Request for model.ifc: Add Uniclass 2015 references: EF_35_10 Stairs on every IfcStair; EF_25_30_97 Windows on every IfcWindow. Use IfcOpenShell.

First a look at what the model holds.

```python
import ifcopenshell

model = ifcopenshell.open("model.ifc")
print(model.schema)
print("classifications:", [c.Name for c in model.by_type("IfcClassification")])
for ifc_class in ("IfcDoor", "IfcRoof", "IfcStair", "IfcWall", "IfcWindow"):
    print(ifc_class, len(model.by_type(ifc_class)))
```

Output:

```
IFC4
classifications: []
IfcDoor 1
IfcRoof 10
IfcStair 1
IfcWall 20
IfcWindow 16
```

```python
import ifcopenshell
import ifcopenshell.api.classification

model = ifcopenshell.open("model.ifc")

system = ifcopenshell.api.classification.add_classification(model, classification="Uniclass 2015")

codes = {
    "IfcStair": ("EF_35_10", "Stairs"),
    "IfcWindow": ("EF_25_30_97", "Windows"),
}
for ifc_class, (code, name) in codes.items():
    products = model.by_type(ifc_class)
    ifcopenshell.api.classification.add_reference(
        model, products=products, classification=system, identification=code, name=name
    )
    print(code, len(products))

model.write("model_updated.ifc")
```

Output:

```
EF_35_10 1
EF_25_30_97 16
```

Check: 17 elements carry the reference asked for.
